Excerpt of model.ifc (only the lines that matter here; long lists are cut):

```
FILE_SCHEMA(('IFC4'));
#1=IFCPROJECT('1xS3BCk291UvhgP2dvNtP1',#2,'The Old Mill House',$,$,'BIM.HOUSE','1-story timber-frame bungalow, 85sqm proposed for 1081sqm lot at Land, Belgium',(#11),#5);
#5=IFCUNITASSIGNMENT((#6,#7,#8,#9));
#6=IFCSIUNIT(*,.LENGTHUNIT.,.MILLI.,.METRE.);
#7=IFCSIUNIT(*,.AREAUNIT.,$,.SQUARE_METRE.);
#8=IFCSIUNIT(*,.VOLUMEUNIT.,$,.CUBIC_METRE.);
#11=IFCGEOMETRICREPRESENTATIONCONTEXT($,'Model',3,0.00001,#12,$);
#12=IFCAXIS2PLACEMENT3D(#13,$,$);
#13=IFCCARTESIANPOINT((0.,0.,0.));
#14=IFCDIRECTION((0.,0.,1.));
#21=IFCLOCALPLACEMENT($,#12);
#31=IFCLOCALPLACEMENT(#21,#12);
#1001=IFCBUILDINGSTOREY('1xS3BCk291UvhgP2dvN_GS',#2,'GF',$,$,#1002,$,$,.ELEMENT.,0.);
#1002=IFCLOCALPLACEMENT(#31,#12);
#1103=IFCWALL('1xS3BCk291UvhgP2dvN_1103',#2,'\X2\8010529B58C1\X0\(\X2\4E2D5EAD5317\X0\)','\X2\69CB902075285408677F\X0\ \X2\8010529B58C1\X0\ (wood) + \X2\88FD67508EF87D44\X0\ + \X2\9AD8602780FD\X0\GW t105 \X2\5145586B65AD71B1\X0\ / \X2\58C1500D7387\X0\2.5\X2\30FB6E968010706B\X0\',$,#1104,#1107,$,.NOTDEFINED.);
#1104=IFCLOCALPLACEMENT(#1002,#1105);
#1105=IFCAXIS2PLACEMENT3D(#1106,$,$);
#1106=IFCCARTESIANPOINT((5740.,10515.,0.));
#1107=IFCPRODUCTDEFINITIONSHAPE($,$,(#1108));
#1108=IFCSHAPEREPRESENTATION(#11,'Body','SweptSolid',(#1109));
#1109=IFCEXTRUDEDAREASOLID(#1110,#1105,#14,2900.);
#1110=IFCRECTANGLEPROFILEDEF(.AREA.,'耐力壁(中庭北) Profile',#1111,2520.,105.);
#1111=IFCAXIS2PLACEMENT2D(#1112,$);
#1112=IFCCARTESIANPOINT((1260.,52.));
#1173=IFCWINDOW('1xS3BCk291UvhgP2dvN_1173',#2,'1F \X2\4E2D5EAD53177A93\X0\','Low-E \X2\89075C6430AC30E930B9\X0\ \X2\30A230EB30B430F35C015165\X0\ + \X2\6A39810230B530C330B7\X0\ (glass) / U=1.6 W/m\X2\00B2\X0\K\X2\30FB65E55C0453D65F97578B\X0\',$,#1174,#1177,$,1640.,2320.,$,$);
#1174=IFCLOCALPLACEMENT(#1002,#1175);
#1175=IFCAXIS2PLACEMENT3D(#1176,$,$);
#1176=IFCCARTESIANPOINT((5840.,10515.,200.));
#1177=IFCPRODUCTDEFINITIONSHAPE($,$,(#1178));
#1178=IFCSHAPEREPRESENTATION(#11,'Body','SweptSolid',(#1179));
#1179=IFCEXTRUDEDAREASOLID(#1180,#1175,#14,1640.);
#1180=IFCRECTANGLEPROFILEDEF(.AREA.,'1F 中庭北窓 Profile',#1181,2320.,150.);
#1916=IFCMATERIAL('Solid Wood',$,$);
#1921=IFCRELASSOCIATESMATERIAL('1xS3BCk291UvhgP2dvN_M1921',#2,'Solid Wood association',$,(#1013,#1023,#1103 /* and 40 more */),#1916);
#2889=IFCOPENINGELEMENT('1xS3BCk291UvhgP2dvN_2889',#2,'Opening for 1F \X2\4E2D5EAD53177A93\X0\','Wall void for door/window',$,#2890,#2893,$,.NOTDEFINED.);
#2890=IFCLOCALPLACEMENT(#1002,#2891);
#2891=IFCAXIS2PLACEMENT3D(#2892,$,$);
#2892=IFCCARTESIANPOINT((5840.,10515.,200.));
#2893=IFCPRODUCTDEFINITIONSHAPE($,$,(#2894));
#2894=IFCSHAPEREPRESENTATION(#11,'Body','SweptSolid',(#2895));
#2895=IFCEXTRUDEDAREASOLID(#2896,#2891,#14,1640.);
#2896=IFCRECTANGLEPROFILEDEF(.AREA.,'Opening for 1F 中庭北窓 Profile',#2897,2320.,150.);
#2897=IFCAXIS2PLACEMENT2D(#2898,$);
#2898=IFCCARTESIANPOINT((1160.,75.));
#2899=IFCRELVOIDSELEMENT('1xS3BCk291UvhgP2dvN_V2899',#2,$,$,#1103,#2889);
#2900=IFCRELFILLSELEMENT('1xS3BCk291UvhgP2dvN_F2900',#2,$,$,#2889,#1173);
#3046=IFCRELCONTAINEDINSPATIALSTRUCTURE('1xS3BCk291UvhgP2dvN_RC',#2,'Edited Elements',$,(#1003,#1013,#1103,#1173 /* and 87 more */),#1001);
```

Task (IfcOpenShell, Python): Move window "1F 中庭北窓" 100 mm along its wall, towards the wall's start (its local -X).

```python
import ifcopenshell
import ifcopenshell.api.geometry
import ifcopenshell.util.placement

model = ifcopenshell.open("model.ifc")

window = model.by_guid("1xS3BCk291UvhgP2dvN_1173")
opening = window.FillsVoids[0].RelatingOpeningElement
wall = opening.VoidsElements[0].RelatingBuildingElement

wall_matrix = ifcopenshell.util.placement.get_local_placement(wall.ObjectPlacement)
shift = wall_matrix[:3, 0] * -100.0
before = ifcopenshell.util.placement.get_local_placement(window.ObjectPlacement)[:3, 3].copy()

# The window is not placed relative to its opening, so move both.
for product in (opening, window):
    matrix = ifcopenshell.util.placement.get_local_placement(product.ObjectPlacement)
    matrix[:3, 3] += shift
    ifcopenshell.api.geometry.edit_object_placement(model, product=product, matrix=matrix, is_si=False)

after = ifcopenshell.util.placement.get_local_placement(window.ObjectPlacement)[:3, 3]
print("window moved by", (after - before).round(3) + 0.0)

model.write("model_edited.ifc")
```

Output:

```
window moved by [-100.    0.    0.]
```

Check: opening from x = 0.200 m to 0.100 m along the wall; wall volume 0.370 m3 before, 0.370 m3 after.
